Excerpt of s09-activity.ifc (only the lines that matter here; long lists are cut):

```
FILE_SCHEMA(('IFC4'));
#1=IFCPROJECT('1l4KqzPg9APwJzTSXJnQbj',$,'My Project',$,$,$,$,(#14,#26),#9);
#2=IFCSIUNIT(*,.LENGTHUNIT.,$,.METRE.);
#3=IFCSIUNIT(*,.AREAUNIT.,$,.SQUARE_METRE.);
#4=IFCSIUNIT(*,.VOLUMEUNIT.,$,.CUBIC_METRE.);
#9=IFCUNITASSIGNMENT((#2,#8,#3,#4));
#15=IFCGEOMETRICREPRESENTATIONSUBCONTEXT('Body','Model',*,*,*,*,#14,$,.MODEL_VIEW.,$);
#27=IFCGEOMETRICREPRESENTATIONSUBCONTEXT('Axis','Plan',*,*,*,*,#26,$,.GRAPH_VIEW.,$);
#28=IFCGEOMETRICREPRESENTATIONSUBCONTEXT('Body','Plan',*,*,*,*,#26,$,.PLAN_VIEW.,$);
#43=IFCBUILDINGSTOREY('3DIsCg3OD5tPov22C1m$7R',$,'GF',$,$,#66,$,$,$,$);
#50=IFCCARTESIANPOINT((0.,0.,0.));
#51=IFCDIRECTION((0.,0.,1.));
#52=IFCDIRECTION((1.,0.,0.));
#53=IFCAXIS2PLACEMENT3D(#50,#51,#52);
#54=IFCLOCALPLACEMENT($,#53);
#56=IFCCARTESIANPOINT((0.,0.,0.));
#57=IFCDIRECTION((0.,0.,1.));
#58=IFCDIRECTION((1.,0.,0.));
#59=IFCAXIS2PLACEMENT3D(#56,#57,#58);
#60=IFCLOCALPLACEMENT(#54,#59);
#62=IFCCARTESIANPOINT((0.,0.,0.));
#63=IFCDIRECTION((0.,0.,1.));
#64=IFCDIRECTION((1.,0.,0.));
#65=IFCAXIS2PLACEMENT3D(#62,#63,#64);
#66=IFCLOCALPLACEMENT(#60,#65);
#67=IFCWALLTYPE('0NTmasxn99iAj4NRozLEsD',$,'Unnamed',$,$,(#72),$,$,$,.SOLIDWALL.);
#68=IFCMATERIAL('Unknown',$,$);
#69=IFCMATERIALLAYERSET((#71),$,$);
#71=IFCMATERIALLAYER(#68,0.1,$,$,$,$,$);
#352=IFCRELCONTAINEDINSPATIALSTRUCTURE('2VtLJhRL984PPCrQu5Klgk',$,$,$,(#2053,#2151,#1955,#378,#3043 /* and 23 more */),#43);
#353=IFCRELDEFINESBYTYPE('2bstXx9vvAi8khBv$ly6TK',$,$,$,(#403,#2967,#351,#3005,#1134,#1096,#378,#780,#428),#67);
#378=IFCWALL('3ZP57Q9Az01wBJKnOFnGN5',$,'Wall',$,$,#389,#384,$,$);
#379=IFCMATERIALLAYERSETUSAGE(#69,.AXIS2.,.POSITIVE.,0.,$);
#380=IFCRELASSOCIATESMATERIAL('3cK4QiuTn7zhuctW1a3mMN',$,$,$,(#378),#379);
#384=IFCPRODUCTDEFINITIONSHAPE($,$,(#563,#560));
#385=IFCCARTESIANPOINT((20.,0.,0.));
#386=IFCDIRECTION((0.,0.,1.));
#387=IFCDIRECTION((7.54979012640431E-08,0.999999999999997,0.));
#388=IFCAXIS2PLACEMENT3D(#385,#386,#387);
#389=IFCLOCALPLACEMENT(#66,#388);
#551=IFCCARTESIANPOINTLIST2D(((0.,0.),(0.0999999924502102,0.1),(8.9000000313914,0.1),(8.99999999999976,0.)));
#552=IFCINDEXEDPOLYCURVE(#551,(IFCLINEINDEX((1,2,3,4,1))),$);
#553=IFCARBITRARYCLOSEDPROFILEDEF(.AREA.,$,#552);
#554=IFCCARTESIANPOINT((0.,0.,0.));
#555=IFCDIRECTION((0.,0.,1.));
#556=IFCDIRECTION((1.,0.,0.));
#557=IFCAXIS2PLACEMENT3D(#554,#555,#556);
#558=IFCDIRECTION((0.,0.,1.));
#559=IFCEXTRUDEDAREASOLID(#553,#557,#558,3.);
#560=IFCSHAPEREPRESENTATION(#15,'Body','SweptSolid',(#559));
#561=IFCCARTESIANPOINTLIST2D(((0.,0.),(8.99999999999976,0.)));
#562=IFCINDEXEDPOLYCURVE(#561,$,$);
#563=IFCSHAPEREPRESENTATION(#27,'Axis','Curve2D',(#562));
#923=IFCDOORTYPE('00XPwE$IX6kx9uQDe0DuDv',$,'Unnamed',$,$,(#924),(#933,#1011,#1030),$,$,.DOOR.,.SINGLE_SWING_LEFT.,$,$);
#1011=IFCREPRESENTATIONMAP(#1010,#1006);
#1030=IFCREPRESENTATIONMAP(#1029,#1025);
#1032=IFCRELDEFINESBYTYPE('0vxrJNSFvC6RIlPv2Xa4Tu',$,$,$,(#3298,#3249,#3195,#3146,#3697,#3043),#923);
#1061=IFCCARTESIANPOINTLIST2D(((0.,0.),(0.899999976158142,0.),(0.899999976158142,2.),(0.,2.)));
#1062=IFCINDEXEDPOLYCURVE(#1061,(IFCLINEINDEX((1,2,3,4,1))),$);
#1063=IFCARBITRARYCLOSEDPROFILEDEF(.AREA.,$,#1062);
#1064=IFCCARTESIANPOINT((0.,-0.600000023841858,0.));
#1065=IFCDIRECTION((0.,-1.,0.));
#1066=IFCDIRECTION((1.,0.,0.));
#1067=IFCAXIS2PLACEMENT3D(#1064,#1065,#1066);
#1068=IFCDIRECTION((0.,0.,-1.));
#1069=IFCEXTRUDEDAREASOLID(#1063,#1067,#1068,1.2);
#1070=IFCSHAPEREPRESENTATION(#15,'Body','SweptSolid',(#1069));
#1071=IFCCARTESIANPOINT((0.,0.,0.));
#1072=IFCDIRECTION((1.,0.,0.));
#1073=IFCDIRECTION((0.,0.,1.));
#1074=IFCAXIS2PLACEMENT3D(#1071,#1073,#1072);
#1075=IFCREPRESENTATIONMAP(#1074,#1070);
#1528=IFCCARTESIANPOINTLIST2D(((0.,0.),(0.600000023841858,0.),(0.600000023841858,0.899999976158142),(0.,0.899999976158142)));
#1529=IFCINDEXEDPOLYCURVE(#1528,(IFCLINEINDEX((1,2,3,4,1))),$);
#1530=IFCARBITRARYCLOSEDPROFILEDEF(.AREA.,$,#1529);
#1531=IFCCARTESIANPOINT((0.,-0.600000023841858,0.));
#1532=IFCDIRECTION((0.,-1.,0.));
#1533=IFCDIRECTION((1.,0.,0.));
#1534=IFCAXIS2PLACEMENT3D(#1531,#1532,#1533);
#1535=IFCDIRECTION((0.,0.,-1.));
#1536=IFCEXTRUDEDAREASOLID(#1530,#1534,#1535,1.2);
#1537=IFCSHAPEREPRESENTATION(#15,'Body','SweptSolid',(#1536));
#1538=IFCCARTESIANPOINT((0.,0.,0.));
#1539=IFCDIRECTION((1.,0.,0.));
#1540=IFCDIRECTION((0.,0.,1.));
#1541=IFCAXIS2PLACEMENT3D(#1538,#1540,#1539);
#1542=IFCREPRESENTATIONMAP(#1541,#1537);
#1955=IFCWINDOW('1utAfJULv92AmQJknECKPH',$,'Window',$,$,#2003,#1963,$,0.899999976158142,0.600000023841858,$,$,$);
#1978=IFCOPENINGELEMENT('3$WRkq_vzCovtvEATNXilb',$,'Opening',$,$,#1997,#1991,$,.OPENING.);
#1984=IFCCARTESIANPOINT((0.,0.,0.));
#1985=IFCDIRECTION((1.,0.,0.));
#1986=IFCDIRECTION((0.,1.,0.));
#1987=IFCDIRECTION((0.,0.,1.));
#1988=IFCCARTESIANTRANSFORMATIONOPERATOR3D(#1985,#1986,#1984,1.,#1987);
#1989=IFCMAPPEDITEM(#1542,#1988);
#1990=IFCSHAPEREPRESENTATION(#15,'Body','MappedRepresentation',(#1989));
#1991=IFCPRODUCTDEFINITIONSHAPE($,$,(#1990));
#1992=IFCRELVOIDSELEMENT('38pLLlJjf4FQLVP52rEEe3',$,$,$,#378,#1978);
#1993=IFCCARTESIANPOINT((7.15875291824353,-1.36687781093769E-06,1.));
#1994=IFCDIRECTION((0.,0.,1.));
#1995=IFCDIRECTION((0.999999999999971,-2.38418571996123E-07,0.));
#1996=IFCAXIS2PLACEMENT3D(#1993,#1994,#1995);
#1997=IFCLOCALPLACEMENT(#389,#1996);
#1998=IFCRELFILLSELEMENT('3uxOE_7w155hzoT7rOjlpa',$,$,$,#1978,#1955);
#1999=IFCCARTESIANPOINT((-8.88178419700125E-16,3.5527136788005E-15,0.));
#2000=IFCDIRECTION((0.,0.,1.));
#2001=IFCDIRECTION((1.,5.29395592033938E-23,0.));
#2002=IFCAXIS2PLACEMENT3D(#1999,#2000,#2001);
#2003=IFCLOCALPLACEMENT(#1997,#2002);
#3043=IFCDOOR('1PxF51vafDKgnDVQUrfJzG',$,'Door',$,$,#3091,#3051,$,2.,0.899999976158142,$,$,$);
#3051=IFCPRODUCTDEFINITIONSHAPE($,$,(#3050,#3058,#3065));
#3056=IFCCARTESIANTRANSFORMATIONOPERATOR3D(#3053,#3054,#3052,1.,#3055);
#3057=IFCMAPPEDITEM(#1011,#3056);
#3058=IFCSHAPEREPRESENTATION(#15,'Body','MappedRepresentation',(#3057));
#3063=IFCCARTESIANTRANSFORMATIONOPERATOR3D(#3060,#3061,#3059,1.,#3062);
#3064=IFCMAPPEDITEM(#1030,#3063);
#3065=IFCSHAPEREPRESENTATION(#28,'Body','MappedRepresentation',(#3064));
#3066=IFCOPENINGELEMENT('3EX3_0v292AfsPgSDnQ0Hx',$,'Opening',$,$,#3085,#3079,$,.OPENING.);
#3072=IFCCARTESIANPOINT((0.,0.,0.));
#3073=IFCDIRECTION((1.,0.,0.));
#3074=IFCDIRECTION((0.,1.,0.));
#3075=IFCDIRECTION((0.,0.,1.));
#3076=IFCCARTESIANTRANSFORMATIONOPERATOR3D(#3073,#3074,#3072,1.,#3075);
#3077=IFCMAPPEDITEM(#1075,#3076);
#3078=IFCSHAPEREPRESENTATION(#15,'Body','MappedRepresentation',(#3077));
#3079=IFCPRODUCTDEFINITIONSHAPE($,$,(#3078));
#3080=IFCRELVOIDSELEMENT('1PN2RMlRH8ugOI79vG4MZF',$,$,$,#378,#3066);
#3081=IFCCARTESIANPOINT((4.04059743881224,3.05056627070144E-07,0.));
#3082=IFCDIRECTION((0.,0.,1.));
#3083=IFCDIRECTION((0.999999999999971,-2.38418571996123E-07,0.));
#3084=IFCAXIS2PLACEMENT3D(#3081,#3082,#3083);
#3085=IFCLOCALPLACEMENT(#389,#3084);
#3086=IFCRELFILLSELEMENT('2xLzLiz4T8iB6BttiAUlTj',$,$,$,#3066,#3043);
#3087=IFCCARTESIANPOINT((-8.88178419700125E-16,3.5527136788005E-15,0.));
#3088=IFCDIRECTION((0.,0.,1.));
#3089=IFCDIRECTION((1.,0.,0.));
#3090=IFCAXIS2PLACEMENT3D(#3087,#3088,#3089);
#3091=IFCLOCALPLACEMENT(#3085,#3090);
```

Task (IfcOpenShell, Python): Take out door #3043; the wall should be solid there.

```python
import ifcopenshell
import ifcopenshell.api.feature
import ifcopenshell.api.root
import ifcopenshell.geom
import ifcopenshell.util.shape

model = ifcopenshell.open("s09-activity.ifc")
settings = ifcopenshell.geom.settings()


def volume(element):
    """Net volume in cubic metres, openings subtracted."""
    shape = ifcopenshell.geom.create_shape(settings, element)
    return ifcopenshell.util.shape.get_volume(shape.geometry)


door = model.by_guid("1PxF51vafDKgnDVQUrfJzG")
opening = door.FillsVoids[0].RelatingOpeningElement
wall = opening.VoidsElements[0].RelatingBuildingElement
before = volume(wall)

ifcopenshell.api.root.remove_product(model, product=door)
ifcopenshell.api.feature.remove_feature(model, feature=opening)

after = volume(wall)

print(f"wall volume {before:.3f} -> {after:.3f} m3")

model.write("s09-activity-out.ifc")
```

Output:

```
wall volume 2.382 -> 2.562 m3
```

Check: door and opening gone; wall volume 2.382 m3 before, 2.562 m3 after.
